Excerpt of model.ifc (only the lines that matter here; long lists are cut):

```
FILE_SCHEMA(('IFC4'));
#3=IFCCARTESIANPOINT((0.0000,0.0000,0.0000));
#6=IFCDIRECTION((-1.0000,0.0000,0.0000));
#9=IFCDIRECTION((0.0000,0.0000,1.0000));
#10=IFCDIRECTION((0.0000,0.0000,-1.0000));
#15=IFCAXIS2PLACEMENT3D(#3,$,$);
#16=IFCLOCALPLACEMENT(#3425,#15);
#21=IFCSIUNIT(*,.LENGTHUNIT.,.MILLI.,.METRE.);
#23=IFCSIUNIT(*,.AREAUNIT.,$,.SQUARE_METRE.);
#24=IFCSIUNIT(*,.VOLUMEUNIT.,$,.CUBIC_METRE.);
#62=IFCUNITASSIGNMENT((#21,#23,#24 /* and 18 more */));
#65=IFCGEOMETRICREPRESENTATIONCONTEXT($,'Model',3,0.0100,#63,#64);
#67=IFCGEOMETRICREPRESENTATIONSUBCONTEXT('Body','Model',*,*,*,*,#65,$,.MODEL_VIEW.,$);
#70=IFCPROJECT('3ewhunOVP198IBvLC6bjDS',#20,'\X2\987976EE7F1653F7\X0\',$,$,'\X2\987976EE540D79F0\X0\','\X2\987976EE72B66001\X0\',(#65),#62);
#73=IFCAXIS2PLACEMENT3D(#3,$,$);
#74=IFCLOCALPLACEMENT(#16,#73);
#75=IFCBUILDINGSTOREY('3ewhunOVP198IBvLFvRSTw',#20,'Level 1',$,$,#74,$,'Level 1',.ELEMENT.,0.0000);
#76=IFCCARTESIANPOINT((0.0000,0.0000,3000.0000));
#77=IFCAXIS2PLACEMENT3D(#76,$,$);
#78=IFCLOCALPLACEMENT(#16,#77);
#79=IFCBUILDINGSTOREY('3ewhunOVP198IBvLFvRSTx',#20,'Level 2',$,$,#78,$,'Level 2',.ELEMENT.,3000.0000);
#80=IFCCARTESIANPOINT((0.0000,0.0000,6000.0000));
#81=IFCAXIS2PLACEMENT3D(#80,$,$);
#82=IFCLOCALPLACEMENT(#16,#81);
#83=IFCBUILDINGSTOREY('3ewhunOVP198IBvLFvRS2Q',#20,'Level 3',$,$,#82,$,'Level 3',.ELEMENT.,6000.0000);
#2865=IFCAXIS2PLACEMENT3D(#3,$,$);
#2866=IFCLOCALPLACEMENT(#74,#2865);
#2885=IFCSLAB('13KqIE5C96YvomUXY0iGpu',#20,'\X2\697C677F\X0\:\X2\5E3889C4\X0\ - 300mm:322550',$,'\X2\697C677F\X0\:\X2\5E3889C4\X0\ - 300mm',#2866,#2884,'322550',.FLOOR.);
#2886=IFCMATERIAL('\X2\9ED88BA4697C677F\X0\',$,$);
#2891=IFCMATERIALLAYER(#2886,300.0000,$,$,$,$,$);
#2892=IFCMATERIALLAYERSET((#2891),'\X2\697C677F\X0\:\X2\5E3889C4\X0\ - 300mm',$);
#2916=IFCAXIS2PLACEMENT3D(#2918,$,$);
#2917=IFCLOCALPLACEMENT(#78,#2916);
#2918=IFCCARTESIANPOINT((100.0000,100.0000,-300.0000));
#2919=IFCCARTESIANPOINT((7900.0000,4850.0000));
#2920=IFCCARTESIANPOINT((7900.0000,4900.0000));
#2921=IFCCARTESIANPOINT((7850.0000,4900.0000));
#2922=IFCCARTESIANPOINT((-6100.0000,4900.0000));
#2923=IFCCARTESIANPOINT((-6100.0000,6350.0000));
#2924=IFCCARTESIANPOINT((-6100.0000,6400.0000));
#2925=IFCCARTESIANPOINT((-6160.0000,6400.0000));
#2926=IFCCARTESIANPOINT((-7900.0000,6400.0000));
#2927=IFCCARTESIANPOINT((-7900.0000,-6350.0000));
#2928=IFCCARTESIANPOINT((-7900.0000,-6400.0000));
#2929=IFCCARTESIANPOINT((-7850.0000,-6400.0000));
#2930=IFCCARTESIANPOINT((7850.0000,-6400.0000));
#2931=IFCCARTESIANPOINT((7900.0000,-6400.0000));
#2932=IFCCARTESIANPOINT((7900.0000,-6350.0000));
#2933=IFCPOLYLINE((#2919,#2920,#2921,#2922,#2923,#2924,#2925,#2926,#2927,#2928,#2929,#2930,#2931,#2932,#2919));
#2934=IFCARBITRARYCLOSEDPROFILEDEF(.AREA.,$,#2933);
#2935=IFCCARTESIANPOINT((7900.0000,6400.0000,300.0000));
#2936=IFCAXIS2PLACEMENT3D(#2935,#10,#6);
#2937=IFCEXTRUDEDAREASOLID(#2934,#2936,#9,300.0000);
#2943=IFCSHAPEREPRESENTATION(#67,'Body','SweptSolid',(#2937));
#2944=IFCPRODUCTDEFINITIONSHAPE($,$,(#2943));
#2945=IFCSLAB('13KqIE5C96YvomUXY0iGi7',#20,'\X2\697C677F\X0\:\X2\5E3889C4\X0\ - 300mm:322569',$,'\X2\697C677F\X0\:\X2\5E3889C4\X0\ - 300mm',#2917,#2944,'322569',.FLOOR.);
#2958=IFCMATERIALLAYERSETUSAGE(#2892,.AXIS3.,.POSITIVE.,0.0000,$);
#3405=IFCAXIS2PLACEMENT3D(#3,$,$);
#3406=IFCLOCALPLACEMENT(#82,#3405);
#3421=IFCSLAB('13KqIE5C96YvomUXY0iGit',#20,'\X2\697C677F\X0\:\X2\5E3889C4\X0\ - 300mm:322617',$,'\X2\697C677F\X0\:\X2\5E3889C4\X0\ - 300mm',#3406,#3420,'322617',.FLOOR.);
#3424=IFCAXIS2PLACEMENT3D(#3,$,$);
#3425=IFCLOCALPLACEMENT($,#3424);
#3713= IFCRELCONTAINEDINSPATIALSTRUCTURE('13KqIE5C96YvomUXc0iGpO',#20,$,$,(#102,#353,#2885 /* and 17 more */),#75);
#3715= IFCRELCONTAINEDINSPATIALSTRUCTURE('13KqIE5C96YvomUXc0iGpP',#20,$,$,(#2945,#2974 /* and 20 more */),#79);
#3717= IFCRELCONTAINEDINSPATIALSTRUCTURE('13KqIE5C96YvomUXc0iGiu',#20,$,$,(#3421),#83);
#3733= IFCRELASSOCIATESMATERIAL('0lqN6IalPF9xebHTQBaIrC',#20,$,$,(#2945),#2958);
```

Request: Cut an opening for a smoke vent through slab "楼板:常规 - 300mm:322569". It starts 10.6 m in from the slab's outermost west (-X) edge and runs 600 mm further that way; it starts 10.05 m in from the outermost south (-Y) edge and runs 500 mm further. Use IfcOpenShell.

```python
import numpy as np
import ifcopenshell
import ifcopenshell.api.feature
import ifcopenshell.api.geometry
import ifcopenshell.api.root
import ifcopenshell.geom
import ifcopenshell.util.placement
import ifcopenshell.util.representation
import ifcopenshell.util.shape
import ifcopenshell.util.unit

model = ifcopenshell.open("model.ifc")
unit_scale = ifcopenshell.util.unit.calculate_unit_scale(model)
settings = ifcopenshell.geom.settings()


def volume(element):
    """Net volume in cubic metres, openings subtracted."""
    shape = ifcopenshell.geom.create_shape(settings, element)
    return ifcopenshell.util.shape.get_volume(shape.geometry)


slab = model.by_guid("13KqIE5C96YvomUXY0iGi7")
before = volume(slab)

# Extent in the slab's own axes, in metres. The edges named are its -X and -Y sides.
slab_shape = ifcopenshell.geom.create_shape(settings, slab)
vertices = ifcopenshell.util.shape.get_vertices(slab_shape.geometry)
x_min, y_min, bottom = vertices.min(axis=0)
top = vertices[:, 2].max()

opening = ifcopenshell.api.root.create_entity(model, ifc_class="IfcOpeningElement", name="Smoke vent opening", predefined_type="OPENING")
context = ifcopenshell.util.representation.get_context(model, "Model", "Body", "MODEL_VIEW")
width, depth = 0.6, 0.5
outline = [(0.0, 0.0), (width, 0.0), (width, depth), (0.0, depth), (0.0, 0.0)]
# Overshoot both faces by 50 mm so the cut is clean.
shape = ifcopenshell.api.geometry.add_slab_representation(
    model, context=context, depth=top - bottom + 0.1, polyline=outline
)
ifcopenshell.api.geometry.assign_representation(model, product=opening, representation=shape)

matrix = ifcopenshell.util.placement.get_local_placement(slab.ObjectPlacement)
matrix[:, 3] = matrix @ np.append(np.array([x_min + 10.6, y_min + 10.05, bottom - 0.05]) / unit_scale, 1.0)
ifcopenshell.api.geometry.edit_object_placement(model, product=opening, matrix=matrix, is_si=False)
ifcopenshell.api.feature.add_feature(model, feature=opening, element=slab)

after = volume(slab)

print(f"slab volume {before:.3f} -> {after:.3f} m3")

model.write("model-out.ifc")
```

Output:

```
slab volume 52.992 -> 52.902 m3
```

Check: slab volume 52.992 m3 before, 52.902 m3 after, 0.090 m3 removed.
